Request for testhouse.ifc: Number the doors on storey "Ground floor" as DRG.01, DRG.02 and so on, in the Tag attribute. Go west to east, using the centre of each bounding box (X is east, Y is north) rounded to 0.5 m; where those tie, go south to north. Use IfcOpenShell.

First a look at what the model holds.

```python
import ifcopenshell
import ifcopenshell.util.element
import ifcopenshell.util.placement

model = ifcopenshell.open("testhouse.ifc")
print(model.schema)
storey = next(s for s in model.by_type("IfcBuildingStorey") if s.Name == "Ground floor")
doors = [e for e in ifcopenshell.util.element.get_decomposition(storey) if e.is_a("IfcDoor")]
for e in sorted(doors, key=lambda e: e.id()):
    origin = ifcopenshell.util.placement.get_local_placement(e.ObjectPlacement)[:3, 3]
    print(e.id(), e.Tag, e.Name, origin.round(2) + 0.0, sep=" | ")
```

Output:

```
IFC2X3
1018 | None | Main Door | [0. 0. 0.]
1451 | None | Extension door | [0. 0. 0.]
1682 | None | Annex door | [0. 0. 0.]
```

```python
import ifcopenshell
import ifcopenshell.geom
import ifcopenshell.util.element
import ifcopenshell.util.shape

model = ifcopenshell.open("testhouse.ifc")
settings = ifcopenshell.geom.settings()
settings.set("use-world-coords", True)


def centre(element):
    shape = ifcopenshell.geom.create_shape(settings, element)
    return ifcopenshell.util.shape.get_bbox_centroid(shape.geometry)


storey = next(s for s in model.by_type("IfcBuildingStorey") if s.Name == "Ground floor")
doors = [e for e in ifcopenshell.util.element.get_decomposition(storey) if e.is_a("IfcDoor")]

# Insertion points can sit at a corner or the storey origin, so sort by the geometry (in metres).
centres = {e: centre(e) for e in doors}
doors.sort(key=lambda e: (round(centres[e][0] / 0.5), centres[e][1]))

for i, e in enumerate(doors, start=1):
    number = f"DRG.{i:02d}"
    e.Tag = number
    print(e.id(), number)

model.write("testhouse-out.ifc")
```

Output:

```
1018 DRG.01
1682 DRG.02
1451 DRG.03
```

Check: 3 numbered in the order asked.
